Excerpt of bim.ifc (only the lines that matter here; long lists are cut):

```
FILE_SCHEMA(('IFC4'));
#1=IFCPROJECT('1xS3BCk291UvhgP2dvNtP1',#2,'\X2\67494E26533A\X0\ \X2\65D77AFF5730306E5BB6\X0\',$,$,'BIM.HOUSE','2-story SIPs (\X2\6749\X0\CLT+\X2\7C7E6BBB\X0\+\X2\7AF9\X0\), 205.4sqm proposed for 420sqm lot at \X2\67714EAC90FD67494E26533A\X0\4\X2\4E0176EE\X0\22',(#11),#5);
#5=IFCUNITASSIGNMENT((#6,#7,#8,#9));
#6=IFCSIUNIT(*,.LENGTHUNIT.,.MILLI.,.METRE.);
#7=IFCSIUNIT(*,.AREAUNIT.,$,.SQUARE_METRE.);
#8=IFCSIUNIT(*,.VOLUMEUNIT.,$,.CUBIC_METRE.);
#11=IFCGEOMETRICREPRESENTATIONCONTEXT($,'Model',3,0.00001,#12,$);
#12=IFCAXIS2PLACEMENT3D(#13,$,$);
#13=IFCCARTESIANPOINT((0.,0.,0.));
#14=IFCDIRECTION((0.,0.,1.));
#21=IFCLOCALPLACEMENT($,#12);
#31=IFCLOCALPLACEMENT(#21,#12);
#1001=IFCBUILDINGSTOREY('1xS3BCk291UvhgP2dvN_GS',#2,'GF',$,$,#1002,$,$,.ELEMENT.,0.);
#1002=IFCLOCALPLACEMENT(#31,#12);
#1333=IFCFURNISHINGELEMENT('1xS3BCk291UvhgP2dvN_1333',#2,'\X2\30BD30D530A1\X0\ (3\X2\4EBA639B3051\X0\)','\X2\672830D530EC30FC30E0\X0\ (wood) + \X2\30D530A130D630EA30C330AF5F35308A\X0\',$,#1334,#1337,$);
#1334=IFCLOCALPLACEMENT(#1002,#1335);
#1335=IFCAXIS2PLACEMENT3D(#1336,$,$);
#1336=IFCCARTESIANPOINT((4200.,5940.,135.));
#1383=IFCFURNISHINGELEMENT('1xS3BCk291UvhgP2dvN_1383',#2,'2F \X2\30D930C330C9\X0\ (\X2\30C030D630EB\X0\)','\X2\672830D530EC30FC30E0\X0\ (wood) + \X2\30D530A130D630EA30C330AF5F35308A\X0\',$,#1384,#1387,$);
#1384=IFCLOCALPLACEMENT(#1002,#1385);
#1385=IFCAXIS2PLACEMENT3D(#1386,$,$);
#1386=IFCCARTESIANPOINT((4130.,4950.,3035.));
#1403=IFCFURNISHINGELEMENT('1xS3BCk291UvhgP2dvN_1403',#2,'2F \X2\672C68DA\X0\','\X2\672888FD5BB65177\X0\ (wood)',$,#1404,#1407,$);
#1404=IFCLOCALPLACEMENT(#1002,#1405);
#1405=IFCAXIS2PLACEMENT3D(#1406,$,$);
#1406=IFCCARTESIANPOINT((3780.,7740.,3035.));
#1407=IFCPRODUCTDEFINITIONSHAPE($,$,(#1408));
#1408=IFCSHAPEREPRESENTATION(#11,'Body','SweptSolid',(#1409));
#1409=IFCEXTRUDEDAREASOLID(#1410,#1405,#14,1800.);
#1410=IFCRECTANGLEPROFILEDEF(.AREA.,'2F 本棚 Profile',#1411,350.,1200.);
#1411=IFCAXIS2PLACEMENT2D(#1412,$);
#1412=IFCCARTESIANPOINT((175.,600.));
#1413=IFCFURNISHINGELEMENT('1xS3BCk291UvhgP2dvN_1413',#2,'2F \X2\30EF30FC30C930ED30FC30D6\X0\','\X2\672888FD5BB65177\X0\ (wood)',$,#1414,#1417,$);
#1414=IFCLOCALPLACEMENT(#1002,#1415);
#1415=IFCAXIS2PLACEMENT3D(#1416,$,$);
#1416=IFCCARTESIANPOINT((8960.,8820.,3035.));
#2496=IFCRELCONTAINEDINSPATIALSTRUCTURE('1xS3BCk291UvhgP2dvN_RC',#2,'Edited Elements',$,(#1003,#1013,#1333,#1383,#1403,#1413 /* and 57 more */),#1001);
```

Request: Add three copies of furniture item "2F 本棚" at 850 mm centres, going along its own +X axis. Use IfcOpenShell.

```python
import ifcopenshell
import ifcopenshell.api.geometry
import ifcopenshell.api.root
import ifcopenshell.util.element
import ifcopenshell.util.placement

model = ifcopenshell.open("bim.ifc")


def reuse_history(source, copy):
    """copy_class also copies each property set's owner history, people and application; keep the originals."""
    for rel in copy.IsDefinedBy:
        if rel.is_a("IfcRelDefinesByProperties") and (history := rel.RelatingPropertyDefinition.OwnerHistory):
            rel.RelatingPropertyDefinition.OwnerHistory = source.OwnerHistory
            ifcopenshell.util.element.remove_deep2(model, history)


source = model.by_guid("1xS3BCk291UvhgP2dvN_1403")
base = ifcopenshell.util.placement.get_local_placement(source.ObjectPlacement)
step = base[:3, 0] * 850.0

for i in range(1, 4):
    copy = ifcopenshell.api.root.copy_class(model, product=source)
    copy.Representation = ifcopenshell.util.element.copy_deep(
        model, source.Representation, exclude=["IfcGeometricRepresentationContext", "IfcRepresentationMap"]
    )
    reuse_history(source, copy)
    matrix = base.copy()
    matrix[:3, 3] += i * step
    print("added at", matrix[:3, 3].round(3) + 0.0)
    ifcopenshell.api.geometry.edit_object_placement(model, product=copy, matrix=matrix, is_si=False)

model.write("bim_edited.ifc")
```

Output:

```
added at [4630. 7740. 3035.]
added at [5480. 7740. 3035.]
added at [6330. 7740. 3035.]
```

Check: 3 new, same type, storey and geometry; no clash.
